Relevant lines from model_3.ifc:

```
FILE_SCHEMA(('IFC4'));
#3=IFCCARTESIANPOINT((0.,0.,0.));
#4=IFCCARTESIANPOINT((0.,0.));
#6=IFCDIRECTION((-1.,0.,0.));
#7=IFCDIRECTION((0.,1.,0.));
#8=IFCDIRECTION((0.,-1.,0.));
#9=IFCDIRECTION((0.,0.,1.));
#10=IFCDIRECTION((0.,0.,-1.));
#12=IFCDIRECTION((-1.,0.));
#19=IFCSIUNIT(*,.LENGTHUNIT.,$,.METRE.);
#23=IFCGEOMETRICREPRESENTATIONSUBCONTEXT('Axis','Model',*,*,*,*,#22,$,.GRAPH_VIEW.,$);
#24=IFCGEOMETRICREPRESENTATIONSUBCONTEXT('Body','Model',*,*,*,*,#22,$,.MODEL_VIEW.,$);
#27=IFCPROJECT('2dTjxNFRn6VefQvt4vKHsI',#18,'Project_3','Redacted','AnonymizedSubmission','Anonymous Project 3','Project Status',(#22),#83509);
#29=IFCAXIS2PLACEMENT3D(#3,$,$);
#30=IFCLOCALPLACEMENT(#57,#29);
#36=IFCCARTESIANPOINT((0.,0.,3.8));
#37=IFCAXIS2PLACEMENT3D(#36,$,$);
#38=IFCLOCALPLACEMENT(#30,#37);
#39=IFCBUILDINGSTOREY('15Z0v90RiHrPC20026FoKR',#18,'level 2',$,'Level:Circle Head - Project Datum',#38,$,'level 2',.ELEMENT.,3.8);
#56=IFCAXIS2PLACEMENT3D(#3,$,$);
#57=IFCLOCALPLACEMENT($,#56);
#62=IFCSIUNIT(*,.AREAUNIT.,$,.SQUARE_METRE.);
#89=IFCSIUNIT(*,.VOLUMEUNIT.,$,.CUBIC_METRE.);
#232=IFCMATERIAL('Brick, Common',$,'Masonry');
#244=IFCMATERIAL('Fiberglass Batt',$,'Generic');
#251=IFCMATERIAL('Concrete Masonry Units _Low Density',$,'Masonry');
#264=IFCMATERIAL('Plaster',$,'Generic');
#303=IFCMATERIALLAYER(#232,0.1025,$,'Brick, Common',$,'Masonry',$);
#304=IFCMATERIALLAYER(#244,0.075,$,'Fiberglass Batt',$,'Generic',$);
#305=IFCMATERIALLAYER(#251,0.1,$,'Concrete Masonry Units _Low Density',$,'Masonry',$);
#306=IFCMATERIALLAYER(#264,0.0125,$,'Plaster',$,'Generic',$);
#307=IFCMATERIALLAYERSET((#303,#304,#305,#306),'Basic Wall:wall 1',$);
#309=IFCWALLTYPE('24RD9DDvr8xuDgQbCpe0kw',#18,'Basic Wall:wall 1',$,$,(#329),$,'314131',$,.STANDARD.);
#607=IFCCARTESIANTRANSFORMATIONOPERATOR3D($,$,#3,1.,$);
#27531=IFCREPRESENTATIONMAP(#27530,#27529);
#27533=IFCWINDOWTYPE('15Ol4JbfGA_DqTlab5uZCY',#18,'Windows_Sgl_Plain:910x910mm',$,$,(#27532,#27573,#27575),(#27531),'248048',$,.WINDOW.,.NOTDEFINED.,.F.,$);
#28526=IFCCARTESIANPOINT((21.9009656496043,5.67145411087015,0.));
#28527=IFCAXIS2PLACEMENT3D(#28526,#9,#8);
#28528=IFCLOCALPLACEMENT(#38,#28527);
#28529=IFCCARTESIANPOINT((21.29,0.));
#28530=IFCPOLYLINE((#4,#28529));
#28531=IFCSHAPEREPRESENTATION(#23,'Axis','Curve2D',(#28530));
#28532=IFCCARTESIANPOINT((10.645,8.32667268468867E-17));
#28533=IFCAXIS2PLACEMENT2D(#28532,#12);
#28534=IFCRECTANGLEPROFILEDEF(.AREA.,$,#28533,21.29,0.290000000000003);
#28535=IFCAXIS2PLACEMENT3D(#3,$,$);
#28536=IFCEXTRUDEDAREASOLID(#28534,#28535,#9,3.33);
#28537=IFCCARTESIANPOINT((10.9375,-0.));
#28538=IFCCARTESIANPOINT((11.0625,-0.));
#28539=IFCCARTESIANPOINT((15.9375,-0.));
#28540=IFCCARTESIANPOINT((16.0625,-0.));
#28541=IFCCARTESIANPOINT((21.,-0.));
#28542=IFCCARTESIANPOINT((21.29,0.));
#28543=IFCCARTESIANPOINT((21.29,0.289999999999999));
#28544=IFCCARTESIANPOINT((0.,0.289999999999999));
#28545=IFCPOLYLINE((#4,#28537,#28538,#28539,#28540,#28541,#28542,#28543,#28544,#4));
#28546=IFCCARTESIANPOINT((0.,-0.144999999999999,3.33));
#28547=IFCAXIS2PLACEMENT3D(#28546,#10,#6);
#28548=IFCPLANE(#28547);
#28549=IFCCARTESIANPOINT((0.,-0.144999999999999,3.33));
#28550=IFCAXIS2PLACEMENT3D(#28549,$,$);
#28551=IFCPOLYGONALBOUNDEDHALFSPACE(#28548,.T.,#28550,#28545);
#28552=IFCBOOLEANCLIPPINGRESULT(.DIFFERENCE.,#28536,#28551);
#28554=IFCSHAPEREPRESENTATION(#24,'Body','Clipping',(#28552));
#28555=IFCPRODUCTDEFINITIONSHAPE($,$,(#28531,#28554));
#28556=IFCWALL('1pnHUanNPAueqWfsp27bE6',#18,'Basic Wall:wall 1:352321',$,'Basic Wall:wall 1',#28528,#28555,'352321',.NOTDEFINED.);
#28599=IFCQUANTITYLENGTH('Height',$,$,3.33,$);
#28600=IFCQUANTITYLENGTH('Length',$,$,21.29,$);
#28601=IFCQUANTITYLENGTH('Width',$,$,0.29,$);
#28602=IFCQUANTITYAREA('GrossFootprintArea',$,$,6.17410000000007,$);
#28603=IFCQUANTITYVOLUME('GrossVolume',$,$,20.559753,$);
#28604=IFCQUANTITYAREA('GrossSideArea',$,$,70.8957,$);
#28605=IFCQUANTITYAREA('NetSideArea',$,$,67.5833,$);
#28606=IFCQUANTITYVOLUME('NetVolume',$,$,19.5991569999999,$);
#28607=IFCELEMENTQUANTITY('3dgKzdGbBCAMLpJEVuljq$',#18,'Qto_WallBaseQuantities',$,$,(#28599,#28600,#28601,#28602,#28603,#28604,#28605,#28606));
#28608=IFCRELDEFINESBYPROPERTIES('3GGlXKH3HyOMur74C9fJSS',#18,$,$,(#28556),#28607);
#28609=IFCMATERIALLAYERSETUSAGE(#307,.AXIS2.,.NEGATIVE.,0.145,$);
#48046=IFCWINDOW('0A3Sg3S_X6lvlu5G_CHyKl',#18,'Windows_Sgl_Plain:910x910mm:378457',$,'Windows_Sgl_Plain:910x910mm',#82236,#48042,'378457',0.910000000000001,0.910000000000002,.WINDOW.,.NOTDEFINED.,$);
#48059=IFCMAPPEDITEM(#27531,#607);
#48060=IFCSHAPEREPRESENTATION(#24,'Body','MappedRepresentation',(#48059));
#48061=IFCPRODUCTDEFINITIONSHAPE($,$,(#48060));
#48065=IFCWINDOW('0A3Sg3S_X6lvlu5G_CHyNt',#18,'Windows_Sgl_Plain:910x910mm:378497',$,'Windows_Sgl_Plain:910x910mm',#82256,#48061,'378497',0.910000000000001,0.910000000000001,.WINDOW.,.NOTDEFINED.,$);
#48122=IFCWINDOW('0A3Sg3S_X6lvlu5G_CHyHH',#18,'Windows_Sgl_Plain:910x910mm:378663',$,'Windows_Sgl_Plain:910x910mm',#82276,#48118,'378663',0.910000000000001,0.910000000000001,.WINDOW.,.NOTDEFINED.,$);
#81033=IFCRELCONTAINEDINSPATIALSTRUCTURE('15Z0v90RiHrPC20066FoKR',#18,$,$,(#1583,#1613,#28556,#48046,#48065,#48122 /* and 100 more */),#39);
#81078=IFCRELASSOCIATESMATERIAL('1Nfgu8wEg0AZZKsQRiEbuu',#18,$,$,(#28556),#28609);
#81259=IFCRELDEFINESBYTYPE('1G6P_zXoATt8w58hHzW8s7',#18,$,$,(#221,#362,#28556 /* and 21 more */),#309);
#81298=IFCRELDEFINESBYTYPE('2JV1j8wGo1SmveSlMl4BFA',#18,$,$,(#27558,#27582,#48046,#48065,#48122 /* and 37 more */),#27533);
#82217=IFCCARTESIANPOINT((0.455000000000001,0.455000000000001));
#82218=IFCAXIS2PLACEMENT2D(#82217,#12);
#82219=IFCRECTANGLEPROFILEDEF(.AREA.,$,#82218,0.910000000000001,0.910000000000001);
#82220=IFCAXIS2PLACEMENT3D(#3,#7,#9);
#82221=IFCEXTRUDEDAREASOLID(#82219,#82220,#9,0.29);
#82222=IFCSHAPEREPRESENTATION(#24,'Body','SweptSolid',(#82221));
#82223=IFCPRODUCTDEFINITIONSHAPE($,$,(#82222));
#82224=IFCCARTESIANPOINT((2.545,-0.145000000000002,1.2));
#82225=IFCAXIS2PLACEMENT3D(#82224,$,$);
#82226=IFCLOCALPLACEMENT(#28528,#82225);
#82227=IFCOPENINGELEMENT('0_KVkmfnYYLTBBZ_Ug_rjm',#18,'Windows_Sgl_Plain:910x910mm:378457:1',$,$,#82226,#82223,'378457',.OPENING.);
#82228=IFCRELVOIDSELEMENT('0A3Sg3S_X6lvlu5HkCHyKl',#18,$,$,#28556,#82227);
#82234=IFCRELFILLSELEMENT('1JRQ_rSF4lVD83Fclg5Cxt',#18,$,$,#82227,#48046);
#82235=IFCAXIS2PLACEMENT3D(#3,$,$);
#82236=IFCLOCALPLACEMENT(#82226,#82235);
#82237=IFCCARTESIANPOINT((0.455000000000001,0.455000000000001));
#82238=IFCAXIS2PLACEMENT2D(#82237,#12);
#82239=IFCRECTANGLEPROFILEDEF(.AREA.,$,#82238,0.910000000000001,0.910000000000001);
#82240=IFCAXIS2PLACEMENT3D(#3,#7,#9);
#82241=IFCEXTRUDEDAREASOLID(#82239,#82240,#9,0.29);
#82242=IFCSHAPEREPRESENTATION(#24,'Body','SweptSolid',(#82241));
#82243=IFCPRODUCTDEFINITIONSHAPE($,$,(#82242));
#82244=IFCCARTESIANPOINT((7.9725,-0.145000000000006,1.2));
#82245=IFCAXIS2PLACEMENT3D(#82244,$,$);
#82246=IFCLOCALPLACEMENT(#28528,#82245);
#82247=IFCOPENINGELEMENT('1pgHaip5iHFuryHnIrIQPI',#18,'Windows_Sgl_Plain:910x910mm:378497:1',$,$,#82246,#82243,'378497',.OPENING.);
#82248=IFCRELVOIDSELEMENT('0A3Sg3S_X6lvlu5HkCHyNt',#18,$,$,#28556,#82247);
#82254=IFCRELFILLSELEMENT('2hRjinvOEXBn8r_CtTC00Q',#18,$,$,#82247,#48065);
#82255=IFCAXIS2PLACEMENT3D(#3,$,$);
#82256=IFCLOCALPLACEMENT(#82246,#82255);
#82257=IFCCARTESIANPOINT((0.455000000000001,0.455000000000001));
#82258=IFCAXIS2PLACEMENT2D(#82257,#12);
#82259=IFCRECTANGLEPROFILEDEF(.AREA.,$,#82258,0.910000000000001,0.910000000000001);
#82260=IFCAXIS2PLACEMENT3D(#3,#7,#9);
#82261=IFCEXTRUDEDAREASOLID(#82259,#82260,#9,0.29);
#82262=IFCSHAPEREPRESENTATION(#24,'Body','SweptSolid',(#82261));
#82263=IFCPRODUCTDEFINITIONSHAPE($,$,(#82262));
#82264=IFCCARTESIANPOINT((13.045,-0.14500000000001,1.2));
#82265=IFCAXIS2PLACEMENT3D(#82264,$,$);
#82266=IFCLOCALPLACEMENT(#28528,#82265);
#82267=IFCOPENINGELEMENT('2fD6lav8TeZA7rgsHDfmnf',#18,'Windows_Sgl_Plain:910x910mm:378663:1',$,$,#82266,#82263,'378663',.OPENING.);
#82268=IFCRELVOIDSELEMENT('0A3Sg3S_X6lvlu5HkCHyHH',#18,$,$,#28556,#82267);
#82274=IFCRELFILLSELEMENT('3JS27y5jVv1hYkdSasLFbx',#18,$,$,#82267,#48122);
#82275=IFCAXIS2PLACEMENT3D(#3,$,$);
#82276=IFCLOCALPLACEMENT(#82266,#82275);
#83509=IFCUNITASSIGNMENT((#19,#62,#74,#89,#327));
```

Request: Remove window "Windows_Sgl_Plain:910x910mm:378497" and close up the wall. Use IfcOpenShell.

```python
import ifcopenshell
import ifcopenshell.api.feature
import ifcopenshell.api.pset
import ifcopenshell.api.root
import ifcopenshell.geom
import ifcopenshell.util.element
import ifcopenshell.util.shape
import ifcopenshell.util.unit

model = ifcopenshell.open("model_3.ifc")
area_scale = ifcopenshell.util.unit.calculate_unit_scale(model, "AREAUNIT")
volume_scale = ifcopenshell.util.unit.calculate_unit_scale(model, "VOLUMEUNIT")
settings = ifcopenshell.geom.settings()


def volume(element):
    """Net volume in cubic metres, openings subtracted."""
    shape = ifcopenshell.geom.create_shape(settings, element)
    return ifcopenshell.util.shape.get_volume(shape.geometry)


window = model.by_guid("0A3Sg3S_X6lvlu5G_CHyNt")
opening = window.FillsVoids[0].RelatingOpeningElement
wall = opening.VoidsElements[0].RelatingBuildingElement
before = volume(wall)

ifcopenshell.api.root.remove_product(model, product=window)
ifcopenshell.api.feature.remove_feature(model, feature=opening)

after = volume(wall)
thickness = 0.29  # wall thickness in metres

# Update the wall's stored quantities.
qto = model.by_id(ifcopenshell.util.element.get_pset(wall, "Qto_WallBaseQuantities", should_inherit=False)["id"])
ifcopenshell.api.pset.edit_qto(model, qto=qto, properties={
    "NetSideArea": after / thickness / area_scale,
    "NetVolume": after / volume_scale,
})

print(f"wall volume {before:.3f} -> {after:.3f} m3")

model.write("model_3_edited.ifc")
```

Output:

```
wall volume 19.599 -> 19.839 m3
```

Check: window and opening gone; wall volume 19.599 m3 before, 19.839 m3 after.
